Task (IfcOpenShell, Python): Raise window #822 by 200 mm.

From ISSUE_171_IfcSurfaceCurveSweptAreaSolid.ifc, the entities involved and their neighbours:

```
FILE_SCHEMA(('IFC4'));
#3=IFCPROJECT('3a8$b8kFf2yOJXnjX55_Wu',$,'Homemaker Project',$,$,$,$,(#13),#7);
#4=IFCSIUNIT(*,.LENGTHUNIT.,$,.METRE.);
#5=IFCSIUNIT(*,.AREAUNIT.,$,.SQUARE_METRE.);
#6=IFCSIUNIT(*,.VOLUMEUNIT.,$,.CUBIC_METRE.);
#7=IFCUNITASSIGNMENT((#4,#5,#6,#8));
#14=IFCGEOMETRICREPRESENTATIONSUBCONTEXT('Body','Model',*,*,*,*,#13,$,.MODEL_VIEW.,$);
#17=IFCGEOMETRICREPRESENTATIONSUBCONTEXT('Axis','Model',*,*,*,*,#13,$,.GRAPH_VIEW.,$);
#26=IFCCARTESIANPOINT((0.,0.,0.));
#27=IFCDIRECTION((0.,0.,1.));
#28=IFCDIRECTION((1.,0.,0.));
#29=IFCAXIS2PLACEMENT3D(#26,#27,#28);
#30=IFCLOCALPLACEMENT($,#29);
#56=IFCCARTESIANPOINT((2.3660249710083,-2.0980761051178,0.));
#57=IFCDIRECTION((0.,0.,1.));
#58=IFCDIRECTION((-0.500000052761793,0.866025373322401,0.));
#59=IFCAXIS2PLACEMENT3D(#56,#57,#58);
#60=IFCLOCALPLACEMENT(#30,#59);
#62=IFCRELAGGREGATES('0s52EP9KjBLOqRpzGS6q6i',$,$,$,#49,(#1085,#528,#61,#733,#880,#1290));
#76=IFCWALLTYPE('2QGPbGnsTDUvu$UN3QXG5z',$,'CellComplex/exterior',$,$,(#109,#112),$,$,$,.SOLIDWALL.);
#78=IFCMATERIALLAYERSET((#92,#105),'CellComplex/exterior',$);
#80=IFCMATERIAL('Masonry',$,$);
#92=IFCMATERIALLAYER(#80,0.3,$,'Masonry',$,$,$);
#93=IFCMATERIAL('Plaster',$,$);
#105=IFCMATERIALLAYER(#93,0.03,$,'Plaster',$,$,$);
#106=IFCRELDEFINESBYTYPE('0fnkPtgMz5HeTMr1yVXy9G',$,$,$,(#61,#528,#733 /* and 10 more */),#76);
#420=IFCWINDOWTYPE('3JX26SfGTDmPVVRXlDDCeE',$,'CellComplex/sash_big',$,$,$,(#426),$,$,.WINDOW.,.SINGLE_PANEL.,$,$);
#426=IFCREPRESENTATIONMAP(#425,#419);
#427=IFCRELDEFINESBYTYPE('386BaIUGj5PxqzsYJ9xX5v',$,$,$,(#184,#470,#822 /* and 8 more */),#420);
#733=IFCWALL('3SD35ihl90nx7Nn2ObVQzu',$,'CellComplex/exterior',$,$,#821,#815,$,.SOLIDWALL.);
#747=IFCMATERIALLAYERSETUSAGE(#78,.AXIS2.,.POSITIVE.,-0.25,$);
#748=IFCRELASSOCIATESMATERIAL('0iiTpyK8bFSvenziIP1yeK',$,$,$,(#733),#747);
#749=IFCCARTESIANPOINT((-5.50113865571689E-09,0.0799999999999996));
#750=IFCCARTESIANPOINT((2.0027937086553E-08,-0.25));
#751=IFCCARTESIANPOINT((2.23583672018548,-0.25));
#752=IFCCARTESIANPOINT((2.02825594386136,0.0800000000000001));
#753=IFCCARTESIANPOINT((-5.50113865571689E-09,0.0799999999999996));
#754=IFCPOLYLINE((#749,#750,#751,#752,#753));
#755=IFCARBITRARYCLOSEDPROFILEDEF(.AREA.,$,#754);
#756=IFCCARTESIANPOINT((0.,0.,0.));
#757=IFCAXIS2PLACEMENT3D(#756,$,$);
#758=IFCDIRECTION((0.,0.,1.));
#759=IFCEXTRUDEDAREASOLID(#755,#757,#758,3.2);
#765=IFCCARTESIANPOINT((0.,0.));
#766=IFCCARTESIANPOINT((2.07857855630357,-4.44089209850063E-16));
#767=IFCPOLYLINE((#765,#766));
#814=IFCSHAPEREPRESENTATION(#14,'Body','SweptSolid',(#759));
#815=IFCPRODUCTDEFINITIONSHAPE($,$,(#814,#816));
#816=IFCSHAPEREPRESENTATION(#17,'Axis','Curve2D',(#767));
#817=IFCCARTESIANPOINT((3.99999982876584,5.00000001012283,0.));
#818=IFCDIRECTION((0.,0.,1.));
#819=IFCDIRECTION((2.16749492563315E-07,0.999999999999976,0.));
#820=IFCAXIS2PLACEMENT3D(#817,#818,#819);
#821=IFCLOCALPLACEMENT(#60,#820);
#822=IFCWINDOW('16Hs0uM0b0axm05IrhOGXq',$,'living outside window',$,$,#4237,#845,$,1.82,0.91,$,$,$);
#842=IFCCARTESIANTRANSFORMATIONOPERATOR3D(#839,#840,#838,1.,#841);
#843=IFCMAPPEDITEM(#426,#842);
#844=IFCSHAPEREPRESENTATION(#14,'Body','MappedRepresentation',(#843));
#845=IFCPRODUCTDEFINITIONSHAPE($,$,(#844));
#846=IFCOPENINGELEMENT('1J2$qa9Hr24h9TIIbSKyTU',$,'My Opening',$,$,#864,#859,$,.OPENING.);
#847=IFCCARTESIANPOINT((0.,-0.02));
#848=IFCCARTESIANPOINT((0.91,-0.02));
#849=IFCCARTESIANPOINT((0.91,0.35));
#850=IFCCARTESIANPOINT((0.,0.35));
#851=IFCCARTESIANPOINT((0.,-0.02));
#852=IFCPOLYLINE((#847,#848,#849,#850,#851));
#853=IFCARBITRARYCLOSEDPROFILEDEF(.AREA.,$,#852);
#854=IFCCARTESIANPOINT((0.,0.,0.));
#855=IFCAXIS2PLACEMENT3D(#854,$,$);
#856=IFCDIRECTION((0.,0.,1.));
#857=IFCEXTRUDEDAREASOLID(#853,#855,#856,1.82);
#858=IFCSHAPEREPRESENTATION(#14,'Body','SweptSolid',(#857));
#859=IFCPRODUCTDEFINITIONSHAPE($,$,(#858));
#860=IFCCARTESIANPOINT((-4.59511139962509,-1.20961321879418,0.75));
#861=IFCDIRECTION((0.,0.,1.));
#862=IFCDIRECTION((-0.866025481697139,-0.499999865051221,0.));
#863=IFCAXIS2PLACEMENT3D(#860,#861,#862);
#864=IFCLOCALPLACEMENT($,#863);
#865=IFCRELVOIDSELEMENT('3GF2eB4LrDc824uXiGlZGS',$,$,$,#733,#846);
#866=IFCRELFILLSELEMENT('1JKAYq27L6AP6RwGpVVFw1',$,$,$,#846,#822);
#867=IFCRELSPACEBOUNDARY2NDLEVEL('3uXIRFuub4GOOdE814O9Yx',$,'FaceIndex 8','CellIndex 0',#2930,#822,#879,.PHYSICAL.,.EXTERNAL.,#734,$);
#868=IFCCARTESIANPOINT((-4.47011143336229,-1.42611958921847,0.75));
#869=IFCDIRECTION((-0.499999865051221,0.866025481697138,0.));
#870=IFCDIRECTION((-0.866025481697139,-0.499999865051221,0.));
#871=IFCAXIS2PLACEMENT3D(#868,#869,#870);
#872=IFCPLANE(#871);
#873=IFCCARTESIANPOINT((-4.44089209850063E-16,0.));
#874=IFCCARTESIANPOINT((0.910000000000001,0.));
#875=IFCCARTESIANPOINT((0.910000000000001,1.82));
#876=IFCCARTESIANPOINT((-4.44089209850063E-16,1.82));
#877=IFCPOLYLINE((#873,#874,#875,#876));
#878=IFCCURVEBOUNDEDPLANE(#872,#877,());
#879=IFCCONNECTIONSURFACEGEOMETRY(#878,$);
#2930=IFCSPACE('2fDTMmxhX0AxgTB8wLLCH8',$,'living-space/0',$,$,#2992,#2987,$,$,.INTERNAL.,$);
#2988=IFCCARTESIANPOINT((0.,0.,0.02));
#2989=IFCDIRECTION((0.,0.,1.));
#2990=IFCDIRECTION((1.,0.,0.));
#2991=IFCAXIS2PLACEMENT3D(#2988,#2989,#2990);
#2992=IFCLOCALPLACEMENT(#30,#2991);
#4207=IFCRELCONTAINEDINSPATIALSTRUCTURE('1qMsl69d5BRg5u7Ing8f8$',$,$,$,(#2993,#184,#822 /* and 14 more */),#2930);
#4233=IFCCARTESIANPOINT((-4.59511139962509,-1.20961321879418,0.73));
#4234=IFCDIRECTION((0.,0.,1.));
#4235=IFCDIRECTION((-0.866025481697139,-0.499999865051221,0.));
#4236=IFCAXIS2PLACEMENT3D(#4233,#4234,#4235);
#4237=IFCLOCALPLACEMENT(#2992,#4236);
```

```python
import numpy as np
import ifcopenshell
import ifcopenshell.api.geometry
import ifcopenshell.util.placement
import ifcopenshell.util.unit

model = ifcopenshell.open("ISSUE_171_IfcSurfaceCurveSweptAreaSolid.ifc")
unit_scale = ifcopenshell.util.unit.calculate_unit_scale(model)

window = model.by_guid("16Hs0uM0b0axm05IrhOGXq")
opening = window.FillsVoids[0].RelatingOpeningElement
dz = 0.2

shift = np.array([0.0, 0.0, dz])
# The window is not placed relative to its opening, so move both.
for product in (opening, window):
    matrix = ifcopenshell.util.placement.get_local_placement(product.ObjectPlacement)
    matrix[:3, 3] += shift
    ifcopenshell.api.geometry.edit_object_placement(model, product=product, matrix=matrix, is_si=False)

# Space boundary surfaces are stored in each space's coordinates; move them too.
for rel in window.ProvidesBoundaries:
    if not rel.ConnectionGeometry:
        continue
    surface = rel.ConnectionGeometry.SurfaceOnRelatingElement.BasisSurface
    space_matrix = ifcopenshell.util.placement.get_local_placement(rel.RelatingSpace.ObjectPlacement)
    point = np.array(surface.Position.Location.Coordinates) + space_matrix[:3, :3].T @ shift
    surface.Position = model.createIfcAxis2Placement3D(
        model.createIfcCartesianPoint(point.tolist()), surface.Position.Axis, surface.Position.RefDirection
    )

print(f"moved by {dz * unit_scale:+.3f} m")

model.write("ISSUE_171_IfcSurfaceCurveSweptAreaSolid_rev.ifc")
```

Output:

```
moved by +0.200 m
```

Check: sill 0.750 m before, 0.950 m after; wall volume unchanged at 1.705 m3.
